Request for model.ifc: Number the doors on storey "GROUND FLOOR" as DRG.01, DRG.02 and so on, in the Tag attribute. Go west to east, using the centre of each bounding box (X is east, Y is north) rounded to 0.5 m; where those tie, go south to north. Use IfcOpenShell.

First a look at what the model holds.

```python
import ifcopenshell
import ifcopenshell.util.element
import ifcopenshell.util.placement

model = ifcopenshell.open("model.ifc")
print(model.schema)
storey = next(s for s in model.by_type("IfcBuildingStorey") if s.Name == "GROUND FLOOR")
doors = [e for e in ifcopenshell.util.element.get_decomposition(storey) if e.is_a("IfcDoor")]
for e in sorted(doors, key=lambda e: e.id()):
    origin = ifcopenshell.util.placement.get_local_placement(e.ObjectPlacement)[:3, 3]
    print(e.id(), e.Tag, e.Name, origin.round(2) + 0.0, sep=" | ")
```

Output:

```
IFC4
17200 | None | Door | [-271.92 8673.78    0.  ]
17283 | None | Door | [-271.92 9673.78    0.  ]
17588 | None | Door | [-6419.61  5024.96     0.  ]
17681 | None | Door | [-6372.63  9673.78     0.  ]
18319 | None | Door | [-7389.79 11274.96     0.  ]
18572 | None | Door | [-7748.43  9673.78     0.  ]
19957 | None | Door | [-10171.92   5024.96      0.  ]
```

```python
import ifcopenshell
import ifcopenshell.geom
import ifcopenshell.util.element
import ifcopenshell.util.shape

model = ifcopenshell.open("model.ifc")
settings = ifcopenshell.geom.settings()
settings.set("use-world-coords", True)


def centre(element):
    shape = ifcopenshell.geom.create_shape(settings, element)
    return ifcopenshell.util.shape.get_bbox_centroid(shape.geometry)


storey = next(s for s in model.by_type("IfcBuildingStorey") if s.Name == "GROUND FLOOR")
doors = [e for e in ifcopenshell.util.element.get_decomposition(storey) if e.is_a("IfcDoor")]

# Insertion points can sit at a corner or the storey origin, so sort by the geometry (in metres).
centres = {e: centre(e) for e in doors}
doors.sort(key=lambda e: (round(centres[e][0] / 0.5), centres[e][1]))

for i, e in enumerate(doors, start=1):
    number = f"DRG.{i:02d}"
    e.Tag = number
    print(e.id(), number)

model.write("model_updated.ifc")
```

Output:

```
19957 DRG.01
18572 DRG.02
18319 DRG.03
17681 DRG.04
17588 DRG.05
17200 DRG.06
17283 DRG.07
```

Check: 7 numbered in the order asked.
